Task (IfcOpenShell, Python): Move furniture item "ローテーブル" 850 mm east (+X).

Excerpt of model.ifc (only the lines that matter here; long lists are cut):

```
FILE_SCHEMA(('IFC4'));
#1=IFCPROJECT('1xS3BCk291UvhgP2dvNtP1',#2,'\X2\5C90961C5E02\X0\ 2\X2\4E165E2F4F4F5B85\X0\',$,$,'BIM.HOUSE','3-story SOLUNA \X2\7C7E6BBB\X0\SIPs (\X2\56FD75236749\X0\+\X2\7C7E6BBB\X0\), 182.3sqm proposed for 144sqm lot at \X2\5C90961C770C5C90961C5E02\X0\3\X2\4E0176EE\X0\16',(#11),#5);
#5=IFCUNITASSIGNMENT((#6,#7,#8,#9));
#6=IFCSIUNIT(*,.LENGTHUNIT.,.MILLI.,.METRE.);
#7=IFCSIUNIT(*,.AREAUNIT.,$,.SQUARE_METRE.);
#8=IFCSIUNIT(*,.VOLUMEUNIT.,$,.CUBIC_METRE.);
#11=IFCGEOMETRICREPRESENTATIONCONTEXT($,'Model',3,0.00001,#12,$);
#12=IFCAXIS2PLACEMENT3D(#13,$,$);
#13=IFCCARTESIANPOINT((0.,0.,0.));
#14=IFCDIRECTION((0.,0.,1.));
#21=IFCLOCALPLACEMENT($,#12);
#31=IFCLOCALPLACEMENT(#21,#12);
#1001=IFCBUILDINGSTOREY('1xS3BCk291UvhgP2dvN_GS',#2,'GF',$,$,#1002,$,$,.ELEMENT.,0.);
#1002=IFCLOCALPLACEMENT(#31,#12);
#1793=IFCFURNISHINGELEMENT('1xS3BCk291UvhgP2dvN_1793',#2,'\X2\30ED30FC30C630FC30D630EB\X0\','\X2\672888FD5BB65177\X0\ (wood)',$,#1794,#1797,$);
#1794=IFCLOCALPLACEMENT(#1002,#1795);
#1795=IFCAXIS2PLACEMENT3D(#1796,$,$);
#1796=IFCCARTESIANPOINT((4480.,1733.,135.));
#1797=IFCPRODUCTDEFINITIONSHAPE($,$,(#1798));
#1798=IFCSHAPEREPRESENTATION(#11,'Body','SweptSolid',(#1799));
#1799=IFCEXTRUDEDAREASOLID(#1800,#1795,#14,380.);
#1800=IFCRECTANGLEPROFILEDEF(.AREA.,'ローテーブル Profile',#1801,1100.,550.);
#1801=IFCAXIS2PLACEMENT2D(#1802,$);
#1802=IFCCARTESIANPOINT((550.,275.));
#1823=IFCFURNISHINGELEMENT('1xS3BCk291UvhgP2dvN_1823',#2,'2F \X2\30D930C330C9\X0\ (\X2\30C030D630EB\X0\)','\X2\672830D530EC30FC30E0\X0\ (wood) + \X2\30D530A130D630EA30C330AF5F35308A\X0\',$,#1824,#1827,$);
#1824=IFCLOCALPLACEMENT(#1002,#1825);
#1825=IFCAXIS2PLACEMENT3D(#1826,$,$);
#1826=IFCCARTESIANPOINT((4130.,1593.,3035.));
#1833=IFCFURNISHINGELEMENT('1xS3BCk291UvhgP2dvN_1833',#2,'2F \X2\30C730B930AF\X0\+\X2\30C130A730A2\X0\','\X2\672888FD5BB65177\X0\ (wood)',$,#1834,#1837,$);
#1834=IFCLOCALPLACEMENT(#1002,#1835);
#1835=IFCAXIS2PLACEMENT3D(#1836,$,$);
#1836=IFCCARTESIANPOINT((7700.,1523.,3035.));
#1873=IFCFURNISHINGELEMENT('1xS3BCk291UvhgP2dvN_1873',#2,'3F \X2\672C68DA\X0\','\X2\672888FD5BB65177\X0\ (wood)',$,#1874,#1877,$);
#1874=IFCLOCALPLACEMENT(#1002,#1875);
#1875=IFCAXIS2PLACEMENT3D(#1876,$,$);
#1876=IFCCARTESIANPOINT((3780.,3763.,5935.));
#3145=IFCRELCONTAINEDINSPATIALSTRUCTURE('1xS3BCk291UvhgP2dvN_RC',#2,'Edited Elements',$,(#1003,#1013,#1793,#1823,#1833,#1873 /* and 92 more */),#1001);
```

```python
import ifcopenshell
import ifcopenshell.api.geometry
import ifcopenshell.util.placement

model = ifcopenshell.open("model.ifc")

item = model.by_guid("1xS3BCk291UvhgP2dvN_1793")
matrix = ifcopenshell.util.placement.get_local_placement(item.ObjectPlacement)
matrix[0, 3] += 850.0
ifcopenshell.api.geometry.edit_object_placement(model, product=item, matrix=matrix, is_si=False)

print(ifcopenshell.util.placement.get_local_placement(item.ObjectPlacement).round(3) + 0.0)

model.write("model_edited.ifc")
```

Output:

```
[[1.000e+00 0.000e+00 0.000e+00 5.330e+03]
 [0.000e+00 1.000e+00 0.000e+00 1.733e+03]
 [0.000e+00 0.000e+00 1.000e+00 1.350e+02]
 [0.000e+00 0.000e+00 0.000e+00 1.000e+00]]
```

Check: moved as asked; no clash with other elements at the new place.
